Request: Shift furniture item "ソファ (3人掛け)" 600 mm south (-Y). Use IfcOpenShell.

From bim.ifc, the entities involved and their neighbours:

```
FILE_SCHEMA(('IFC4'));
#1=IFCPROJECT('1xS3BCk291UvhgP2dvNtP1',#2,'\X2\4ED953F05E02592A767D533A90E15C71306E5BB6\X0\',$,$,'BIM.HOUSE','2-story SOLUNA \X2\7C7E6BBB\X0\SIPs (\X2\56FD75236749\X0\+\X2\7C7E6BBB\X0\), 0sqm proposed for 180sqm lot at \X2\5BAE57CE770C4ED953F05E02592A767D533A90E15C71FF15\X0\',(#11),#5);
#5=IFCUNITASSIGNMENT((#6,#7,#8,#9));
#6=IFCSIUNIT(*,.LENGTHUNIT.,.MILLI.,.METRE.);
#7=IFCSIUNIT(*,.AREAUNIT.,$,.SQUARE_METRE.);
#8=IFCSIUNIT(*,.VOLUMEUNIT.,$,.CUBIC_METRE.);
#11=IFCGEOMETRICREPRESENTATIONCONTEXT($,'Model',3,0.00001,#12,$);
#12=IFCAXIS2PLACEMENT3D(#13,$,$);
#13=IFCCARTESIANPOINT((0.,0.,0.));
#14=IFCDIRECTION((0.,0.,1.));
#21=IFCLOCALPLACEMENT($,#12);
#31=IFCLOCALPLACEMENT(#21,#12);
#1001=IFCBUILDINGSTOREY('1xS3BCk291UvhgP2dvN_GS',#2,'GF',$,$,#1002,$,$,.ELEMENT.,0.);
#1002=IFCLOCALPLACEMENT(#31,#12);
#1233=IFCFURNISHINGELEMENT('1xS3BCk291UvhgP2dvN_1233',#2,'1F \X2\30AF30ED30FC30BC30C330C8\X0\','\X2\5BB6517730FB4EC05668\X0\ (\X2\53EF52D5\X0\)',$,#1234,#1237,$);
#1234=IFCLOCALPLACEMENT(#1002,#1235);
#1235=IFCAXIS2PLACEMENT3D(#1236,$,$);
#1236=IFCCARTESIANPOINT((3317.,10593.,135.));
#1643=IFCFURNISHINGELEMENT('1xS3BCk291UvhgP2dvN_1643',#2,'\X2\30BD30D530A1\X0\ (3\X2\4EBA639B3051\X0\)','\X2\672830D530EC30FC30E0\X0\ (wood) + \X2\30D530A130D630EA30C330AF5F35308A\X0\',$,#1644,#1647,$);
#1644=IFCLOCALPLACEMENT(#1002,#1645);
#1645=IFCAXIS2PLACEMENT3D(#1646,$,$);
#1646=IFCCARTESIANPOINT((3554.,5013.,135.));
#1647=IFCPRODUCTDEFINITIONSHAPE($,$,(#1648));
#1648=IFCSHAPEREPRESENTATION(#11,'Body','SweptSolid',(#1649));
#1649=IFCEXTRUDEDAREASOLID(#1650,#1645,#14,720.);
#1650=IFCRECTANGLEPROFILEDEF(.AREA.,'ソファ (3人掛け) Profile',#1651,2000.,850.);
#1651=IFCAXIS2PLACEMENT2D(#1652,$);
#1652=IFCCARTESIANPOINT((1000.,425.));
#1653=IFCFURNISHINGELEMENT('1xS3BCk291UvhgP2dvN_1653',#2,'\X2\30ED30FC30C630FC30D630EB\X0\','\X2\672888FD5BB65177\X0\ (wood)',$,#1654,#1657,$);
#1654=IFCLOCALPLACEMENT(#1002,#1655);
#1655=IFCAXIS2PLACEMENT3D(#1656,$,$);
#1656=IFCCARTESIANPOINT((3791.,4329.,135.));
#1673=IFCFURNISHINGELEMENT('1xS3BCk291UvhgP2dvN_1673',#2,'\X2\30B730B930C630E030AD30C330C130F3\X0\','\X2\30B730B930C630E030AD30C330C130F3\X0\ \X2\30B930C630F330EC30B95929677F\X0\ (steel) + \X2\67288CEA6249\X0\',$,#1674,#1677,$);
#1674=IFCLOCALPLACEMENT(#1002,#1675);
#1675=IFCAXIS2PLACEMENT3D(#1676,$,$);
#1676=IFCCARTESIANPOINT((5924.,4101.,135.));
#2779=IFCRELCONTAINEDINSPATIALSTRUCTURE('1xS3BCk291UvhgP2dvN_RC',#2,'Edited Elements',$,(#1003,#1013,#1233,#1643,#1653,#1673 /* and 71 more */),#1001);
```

```python
import ifcopenshell
import ifcopenshell.api.geometry
import ifcopenshell.util.placement

model = ifcopenshell.open("bim.ifc")

item = model.by_guid("1xS3BCk291UvhgP2dvN_1643")
matrix = ifcopenshell.util.placement.get_local_placement(item.ObjectPlacement)
matrix[1, 3] -= 600.0
ifcopenshell.api.geometry.edit_object_placement(model, product=item, matrix=matrix, is_si=False)

print(ifcopenshell.util.placement.get_local_placement(item.ObjectPlacement).round(3) + 0.0)

model.write("bim-out.ifc")
```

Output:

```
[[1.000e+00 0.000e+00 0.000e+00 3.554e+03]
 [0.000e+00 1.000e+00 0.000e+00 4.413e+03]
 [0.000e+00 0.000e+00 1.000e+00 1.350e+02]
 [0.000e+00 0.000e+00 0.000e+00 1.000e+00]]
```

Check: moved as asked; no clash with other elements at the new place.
